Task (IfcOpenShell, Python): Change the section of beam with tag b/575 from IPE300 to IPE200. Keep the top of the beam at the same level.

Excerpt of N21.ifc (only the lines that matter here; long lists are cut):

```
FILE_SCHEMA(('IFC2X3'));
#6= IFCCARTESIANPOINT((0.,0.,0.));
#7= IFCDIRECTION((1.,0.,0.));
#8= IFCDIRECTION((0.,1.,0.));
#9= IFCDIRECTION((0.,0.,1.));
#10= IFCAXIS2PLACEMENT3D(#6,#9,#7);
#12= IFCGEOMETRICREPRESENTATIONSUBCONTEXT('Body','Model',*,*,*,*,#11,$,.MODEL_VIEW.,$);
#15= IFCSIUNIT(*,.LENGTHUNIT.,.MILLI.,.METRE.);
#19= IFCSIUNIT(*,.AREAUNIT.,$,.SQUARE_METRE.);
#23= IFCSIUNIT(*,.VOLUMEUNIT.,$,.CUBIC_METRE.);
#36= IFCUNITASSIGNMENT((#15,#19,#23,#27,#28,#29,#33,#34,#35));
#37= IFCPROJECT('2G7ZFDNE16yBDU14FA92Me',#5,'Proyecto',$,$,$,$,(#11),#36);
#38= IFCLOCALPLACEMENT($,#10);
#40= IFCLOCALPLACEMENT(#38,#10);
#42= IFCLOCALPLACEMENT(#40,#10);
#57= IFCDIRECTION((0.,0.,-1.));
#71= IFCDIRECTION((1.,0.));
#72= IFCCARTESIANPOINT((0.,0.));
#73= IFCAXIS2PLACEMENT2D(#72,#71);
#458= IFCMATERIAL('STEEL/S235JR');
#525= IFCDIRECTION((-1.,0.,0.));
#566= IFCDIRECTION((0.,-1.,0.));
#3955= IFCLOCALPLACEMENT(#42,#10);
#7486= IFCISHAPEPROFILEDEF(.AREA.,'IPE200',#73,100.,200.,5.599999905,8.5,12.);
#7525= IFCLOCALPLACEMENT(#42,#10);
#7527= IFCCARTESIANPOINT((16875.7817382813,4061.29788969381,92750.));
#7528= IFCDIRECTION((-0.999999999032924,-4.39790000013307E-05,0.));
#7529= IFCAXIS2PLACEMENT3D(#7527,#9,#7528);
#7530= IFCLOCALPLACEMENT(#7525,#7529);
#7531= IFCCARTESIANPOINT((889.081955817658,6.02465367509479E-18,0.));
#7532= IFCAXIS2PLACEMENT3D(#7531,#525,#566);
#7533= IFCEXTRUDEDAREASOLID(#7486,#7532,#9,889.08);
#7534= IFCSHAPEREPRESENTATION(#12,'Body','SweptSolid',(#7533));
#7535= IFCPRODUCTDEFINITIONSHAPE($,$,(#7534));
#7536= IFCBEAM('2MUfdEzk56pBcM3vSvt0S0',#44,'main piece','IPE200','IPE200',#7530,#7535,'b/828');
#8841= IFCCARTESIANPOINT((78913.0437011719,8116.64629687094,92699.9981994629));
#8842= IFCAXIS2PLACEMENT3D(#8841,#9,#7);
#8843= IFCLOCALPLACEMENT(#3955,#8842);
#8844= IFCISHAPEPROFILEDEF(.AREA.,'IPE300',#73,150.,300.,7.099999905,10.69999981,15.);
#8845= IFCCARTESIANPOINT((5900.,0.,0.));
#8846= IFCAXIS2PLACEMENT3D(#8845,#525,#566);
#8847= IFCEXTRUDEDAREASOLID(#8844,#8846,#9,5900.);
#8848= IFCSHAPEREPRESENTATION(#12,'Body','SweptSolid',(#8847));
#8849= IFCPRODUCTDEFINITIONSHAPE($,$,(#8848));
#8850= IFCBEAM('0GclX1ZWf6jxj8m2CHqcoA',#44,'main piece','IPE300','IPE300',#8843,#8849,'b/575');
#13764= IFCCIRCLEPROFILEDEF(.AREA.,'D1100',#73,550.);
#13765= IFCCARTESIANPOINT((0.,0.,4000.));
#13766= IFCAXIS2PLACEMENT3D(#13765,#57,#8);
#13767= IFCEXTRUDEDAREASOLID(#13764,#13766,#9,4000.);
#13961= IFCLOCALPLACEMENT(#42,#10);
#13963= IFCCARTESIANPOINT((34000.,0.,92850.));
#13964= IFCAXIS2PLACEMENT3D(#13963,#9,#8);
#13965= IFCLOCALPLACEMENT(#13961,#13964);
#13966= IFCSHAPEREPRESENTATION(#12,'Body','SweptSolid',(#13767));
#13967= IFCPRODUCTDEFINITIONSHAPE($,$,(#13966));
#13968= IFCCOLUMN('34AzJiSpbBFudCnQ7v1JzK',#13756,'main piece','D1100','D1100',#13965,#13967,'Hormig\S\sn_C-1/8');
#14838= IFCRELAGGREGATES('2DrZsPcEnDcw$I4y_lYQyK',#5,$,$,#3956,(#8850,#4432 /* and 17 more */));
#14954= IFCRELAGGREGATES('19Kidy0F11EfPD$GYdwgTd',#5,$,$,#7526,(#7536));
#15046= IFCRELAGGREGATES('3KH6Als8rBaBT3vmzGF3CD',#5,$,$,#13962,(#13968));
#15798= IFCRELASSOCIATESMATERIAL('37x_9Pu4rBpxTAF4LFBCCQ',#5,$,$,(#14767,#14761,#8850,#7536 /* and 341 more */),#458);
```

```python
import ifcopenshell
import ifcopenshell.util.element
import ifcopenshell.util.representation

model = ifcopenshell.open("N21.ifc")

member = model.by_guid("0GclX1ZWf6jxj8m2CHqcoA")
source = next(p for p in model.by_type("IfcIShapeProfileDef") if p.ProfileName == "IPE200")

body = ifcopenshell.util.representation.get_representation(member, "Model", "Body")
solid = body.Items[0]
old_profile = solid.SweptArea

# Copy the section's sizes but keep this member's own profile position.
profile = ifcopenshell.util.element.copy(model, source)
# Profiles are centred, so shift by half the change in depth to hold the top.
shift = (old_profile.OverallDepth - profile.OverallDepth) / 2
x, y = old_profile.Position.Location.Coordinates
up = (0.0, 1.0)  # upwards, in the solid's own plane
location = model.createIfcCartesianPoint((x + up[0] * shift, y + up[1] * shift))
profile.Position = model.createIfcAxis2Placement2D(location, old_profile.Position.RefDirection)
solid.SweptArea = profile
if not model.get_total_inverses(old_profile):
    ifcopenshell.util.element.remove_deep2(model, old_profile)
member.Description = member.Description.replace("IPE300", "IPE200")
member.ObjectType = member.ObjectType.replace("IPE300", "IPE200")

print(solid.SweptArea)

model.write("N21_edited.ifc")
```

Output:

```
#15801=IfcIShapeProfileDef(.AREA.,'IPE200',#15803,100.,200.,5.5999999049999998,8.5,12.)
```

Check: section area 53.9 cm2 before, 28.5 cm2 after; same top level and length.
